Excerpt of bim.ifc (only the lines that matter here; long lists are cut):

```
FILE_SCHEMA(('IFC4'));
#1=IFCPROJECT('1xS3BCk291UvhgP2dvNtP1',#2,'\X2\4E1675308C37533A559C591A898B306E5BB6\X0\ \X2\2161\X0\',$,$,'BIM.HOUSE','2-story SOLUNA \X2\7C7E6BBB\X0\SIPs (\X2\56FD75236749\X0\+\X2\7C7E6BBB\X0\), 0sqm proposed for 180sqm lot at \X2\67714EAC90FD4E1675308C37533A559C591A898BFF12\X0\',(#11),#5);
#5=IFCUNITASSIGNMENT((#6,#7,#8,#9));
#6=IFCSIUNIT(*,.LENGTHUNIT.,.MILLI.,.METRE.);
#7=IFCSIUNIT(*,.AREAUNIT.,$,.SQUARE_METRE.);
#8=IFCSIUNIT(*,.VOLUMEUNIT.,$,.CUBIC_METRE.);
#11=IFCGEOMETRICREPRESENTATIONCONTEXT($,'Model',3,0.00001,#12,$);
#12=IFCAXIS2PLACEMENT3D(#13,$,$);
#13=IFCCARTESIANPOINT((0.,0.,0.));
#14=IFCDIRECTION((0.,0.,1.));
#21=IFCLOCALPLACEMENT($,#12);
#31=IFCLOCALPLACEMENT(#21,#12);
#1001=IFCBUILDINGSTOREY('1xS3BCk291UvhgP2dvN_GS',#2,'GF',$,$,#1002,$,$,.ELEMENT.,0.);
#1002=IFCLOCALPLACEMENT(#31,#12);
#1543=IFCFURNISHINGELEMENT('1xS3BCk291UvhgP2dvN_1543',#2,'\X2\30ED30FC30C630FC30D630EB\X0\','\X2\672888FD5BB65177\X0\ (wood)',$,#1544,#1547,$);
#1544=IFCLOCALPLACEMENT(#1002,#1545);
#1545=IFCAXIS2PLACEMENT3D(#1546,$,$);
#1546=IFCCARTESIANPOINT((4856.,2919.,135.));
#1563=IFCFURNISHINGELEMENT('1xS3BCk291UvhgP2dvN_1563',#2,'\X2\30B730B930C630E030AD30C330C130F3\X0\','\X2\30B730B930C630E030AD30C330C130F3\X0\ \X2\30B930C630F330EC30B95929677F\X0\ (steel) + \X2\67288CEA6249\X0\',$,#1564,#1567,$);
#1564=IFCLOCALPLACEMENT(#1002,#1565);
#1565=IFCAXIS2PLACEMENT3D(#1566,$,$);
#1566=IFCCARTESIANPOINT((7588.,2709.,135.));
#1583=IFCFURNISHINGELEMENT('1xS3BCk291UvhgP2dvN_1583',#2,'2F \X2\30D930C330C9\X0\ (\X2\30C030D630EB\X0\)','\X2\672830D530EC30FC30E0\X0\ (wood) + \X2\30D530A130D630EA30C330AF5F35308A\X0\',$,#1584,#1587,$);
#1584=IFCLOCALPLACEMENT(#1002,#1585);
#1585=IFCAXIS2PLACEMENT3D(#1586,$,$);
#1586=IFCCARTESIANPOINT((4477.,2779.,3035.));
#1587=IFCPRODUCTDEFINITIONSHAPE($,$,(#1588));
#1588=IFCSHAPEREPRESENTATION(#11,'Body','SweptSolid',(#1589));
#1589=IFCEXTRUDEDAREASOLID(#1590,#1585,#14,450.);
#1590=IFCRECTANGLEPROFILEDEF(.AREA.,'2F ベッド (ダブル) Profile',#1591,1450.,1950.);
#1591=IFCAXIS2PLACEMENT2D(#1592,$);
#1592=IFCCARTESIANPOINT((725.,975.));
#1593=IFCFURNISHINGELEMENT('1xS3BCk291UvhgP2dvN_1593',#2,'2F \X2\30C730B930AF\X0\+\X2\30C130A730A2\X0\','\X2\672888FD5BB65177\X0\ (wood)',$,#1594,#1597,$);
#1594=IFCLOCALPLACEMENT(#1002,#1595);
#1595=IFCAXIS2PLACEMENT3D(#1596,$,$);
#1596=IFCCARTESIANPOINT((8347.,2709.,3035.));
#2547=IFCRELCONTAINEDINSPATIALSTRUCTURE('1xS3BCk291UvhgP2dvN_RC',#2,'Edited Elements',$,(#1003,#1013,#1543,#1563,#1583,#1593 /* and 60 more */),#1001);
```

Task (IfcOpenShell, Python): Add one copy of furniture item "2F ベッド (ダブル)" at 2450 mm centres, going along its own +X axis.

```python
import ifcopenshell
import ifcopenshell.api.geometry
import ifcopenshell.api.root
import ifcopenshell.util.element
import ifcopenshell.util.placement
import ifcopenshell.util.unit

model = ifcopenshell.open("bim.ifc")
unit_scale = ifcopenshell.util.unit.calculate_unit_scale(model)


def reuse_history(source, copy):
    """copy_class also copies each property set's owner history, people and application; keep the originals."""
    for rel in copy.IsDefinedBy:
        if rel.is_a("IfcRelDefinesByProperties") and (history := rel.RelatingPropertyDefinition.OwnerHistory):
            rel.RelatingPropertyDefinition.OwnerHistory = source.OwnerHistory
            ifcopenshell.util.element.remove_deep2(model, history)


source = model.by_id(1583)
base = ifcopenshell.util.placement.get_local_placement(source.ObjectPlacement)
step = base[:3, 0] * 2.45 / unit_scale

for i in range(1, 2):
    copy = ifcopenshell.api.root.copy_class(model, product=source)
    copy.Representation = ifcopenshell.util.element.copy_deep(
        model, source.Representation, exclude=["IfcGeometricRepresentationContext", "IfcRepresentationMap"]
    )
    reuse_history(source, copy)
    matrix = base.copy()
    matrix[:3, 3] += i * step
    print("added at", matrix[:3, 3].round(3) + 0.0)
    ifcopenshell.api.geometry.edit_object_placement(model, product=copy, matrix=matrix, is_si=False)

model.write("bim_edited.ifc")
```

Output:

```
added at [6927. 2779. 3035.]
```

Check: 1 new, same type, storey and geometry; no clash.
